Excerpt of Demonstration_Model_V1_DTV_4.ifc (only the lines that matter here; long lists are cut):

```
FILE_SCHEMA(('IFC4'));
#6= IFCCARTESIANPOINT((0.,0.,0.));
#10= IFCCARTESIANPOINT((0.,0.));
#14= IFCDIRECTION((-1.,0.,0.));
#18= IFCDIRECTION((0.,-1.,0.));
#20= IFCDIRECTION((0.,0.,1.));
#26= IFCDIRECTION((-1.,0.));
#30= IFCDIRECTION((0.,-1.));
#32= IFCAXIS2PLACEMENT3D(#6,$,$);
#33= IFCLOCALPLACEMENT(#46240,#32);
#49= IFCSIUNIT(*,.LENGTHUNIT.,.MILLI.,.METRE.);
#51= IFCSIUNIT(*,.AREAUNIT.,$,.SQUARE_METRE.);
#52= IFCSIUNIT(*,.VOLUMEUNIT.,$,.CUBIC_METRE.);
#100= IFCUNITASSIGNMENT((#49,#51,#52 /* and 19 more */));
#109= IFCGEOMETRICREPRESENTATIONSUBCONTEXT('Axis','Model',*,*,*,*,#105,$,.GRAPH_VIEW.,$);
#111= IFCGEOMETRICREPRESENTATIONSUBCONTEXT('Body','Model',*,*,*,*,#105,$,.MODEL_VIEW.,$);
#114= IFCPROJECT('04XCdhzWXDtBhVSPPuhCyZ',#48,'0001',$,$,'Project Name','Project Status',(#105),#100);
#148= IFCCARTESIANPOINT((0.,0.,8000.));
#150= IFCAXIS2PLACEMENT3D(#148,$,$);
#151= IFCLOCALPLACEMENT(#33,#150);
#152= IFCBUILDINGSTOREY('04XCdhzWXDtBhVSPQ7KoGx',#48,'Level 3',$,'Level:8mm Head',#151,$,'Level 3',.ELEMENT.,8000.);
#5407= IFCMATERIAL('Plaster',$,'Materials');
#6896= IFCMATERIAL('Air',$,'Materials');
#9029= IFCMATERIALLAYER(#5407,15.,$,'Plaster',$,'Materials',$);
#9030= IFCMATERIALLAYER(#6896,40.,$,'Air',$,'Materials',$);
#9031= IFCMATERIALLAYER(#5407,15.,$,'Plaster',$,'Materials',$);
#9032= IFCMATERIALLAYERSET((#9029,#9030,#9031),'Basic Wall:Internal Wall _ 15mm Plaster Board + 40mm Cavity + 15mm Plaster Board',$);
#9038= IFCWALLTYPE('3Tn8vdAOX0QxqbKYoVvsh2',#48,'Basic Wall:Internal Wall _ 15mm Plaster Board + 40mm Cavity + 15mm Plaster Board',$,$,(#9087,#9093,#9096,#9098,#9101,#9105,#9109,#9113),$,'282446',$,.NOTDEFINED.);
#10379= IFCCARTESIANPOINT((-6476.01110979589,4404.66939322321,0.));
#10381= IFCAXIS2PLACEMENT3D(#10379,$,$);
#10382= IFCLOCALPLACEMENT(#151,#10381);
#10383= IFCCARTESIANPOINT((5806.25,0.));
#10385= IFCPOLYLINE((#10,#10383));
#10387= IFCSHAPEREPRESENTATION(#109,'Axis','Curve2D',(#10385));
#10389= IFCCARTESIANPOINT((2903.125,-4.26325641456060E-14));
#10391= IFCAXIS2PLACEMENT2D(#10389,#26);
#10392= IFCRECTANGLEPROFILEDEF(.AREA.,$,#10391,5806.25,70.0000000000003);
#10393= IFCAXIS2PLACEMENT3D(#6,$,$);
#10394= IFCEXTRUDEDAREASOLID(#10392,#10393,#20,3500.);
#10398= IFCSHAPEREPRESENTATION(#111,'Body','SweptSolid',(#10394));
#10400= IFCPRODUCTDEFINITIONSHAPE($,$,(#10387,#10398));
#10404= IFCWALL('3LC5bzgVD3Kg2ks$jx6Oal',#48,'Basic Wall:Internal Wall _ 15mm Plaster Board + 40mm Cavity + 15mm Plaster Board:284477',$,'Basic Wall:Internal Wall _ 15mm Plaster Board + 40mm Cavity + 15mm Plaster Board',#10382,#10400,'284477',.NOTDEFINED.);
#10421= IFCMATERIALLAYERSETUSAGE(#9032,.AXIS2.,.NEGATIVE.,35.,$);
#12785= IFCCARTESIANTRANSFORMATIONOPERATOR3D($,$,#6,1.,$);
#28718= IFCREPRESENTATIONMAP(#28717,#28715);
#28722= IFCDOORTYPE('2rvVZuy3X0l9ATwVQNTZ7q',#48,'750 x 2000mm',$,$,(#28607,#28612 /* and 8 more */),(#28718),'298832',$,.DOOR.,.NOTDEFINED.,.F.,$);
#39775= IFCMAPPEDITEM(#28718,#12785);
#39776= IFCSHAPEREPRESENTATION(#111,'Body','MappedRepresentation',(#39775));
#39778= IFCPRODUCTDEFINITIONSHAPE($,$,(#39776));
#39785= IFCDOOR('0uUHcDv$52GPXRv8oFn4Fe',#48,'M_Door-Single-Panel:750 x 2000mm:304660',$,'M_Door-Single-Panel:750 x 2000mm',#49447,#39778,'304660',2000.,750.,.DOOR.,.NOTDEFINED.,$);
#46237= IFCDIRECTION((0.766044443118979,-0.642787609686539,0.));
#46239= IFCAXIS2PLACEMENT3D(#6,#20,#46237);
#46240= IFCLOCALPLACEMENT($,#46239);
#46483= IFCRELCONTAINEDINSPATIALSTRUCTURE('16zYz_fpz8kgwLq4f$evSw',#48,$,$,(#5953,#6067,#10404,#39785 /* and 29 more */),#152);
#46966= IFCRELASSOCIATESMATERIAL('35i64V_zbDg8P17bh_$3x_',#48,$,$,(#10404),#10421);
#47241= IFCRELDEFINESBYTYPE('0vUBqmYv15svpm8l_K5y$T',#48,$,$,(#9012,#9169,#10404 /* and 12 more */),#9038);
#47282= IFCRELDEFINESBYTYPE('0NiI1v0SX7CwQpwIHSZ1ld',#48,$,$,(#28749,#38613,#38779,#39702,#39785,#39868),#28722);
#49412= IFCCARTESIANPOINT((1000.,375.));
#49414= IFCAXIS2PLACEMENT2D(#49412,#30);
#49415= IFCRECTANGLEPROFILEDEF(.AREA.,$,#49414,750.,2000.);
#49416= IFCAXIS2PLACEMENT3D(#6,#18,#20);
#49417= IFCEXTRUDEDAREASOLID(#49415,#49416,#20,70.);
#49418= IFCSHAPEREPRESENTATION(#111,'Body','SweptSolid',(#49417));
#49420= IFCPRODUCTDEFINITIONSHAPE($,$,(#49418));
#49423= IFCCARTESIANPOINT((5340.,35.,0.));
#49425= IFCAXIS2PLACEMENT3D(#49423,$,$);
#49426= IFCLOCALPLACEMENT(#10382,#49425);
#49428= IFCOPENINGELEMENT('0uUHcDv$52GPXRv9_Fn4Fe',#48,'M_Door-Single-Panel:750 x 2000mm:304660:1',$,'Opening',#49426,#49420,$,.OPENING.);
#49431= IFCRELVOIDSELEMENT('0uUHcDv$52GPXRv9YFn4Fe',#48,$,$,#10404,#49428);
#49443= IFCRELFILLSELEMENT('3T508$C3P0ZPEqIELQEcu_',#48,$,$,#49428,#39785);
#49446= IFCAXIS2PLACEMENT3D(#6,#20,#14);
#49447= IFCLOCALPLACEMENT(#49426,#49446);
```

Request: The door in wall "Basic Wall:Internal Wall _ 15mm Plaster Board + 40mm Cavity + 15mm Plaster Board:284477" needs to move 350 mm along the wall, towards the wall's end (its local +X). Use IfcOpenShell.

```python
import ifcopenshell
import ifcopenshell.api.geometry
import ifcopenshell.util.placement
import ifcopenshell.util.unit

model = ifcopenshell.open("Demonstration_Model_V1_DTV_4.ifc")
unit_scale = ifcopenshell.util.unit.calculate_unit_scale(model)

door = model.by_guid("0uUHcDv$52GPXRv8oFn4Fe")
opening = door.FillsVoids[0].RelatingOpeningElement
wall = opening.VoidsElements[0].RelatingBuildingElement

wall_matrix = ifcopenshell.util.placement.get_local_placement(wall.ObjectPlacement)
shift = wall_matrix[:3, 0] * 0.35 / unit_scale
before = ifcopenshell.util.placement.get_local_placement(door.ObjectPlacement)[:3, 3].copy()

# The door is placed relative to its opening, so it follows when the opening moves.
matrix = ifcopenshell.util.placement.get_local_placement(opening.ObjectPlacement)
matrix[:3, 3] += shift
ifcopenshell.api.geometry.edit_object_placement(
    model, product=opening, matrix=matrix, is_si=False, should_transform_children=True
)

after = ifcopenshell.util.placement.get_local_placement(door.ObjectPlacement)[:3, 3]
print("door moved by", (after - before).round(3) + 0.0)

model.write("Demonstration_Model_V1_DTV_4_updated.ifc")
```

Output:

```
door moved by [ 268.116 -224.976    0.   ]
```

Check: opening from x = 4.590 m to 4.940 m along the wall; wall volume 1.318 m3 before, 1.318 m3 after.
